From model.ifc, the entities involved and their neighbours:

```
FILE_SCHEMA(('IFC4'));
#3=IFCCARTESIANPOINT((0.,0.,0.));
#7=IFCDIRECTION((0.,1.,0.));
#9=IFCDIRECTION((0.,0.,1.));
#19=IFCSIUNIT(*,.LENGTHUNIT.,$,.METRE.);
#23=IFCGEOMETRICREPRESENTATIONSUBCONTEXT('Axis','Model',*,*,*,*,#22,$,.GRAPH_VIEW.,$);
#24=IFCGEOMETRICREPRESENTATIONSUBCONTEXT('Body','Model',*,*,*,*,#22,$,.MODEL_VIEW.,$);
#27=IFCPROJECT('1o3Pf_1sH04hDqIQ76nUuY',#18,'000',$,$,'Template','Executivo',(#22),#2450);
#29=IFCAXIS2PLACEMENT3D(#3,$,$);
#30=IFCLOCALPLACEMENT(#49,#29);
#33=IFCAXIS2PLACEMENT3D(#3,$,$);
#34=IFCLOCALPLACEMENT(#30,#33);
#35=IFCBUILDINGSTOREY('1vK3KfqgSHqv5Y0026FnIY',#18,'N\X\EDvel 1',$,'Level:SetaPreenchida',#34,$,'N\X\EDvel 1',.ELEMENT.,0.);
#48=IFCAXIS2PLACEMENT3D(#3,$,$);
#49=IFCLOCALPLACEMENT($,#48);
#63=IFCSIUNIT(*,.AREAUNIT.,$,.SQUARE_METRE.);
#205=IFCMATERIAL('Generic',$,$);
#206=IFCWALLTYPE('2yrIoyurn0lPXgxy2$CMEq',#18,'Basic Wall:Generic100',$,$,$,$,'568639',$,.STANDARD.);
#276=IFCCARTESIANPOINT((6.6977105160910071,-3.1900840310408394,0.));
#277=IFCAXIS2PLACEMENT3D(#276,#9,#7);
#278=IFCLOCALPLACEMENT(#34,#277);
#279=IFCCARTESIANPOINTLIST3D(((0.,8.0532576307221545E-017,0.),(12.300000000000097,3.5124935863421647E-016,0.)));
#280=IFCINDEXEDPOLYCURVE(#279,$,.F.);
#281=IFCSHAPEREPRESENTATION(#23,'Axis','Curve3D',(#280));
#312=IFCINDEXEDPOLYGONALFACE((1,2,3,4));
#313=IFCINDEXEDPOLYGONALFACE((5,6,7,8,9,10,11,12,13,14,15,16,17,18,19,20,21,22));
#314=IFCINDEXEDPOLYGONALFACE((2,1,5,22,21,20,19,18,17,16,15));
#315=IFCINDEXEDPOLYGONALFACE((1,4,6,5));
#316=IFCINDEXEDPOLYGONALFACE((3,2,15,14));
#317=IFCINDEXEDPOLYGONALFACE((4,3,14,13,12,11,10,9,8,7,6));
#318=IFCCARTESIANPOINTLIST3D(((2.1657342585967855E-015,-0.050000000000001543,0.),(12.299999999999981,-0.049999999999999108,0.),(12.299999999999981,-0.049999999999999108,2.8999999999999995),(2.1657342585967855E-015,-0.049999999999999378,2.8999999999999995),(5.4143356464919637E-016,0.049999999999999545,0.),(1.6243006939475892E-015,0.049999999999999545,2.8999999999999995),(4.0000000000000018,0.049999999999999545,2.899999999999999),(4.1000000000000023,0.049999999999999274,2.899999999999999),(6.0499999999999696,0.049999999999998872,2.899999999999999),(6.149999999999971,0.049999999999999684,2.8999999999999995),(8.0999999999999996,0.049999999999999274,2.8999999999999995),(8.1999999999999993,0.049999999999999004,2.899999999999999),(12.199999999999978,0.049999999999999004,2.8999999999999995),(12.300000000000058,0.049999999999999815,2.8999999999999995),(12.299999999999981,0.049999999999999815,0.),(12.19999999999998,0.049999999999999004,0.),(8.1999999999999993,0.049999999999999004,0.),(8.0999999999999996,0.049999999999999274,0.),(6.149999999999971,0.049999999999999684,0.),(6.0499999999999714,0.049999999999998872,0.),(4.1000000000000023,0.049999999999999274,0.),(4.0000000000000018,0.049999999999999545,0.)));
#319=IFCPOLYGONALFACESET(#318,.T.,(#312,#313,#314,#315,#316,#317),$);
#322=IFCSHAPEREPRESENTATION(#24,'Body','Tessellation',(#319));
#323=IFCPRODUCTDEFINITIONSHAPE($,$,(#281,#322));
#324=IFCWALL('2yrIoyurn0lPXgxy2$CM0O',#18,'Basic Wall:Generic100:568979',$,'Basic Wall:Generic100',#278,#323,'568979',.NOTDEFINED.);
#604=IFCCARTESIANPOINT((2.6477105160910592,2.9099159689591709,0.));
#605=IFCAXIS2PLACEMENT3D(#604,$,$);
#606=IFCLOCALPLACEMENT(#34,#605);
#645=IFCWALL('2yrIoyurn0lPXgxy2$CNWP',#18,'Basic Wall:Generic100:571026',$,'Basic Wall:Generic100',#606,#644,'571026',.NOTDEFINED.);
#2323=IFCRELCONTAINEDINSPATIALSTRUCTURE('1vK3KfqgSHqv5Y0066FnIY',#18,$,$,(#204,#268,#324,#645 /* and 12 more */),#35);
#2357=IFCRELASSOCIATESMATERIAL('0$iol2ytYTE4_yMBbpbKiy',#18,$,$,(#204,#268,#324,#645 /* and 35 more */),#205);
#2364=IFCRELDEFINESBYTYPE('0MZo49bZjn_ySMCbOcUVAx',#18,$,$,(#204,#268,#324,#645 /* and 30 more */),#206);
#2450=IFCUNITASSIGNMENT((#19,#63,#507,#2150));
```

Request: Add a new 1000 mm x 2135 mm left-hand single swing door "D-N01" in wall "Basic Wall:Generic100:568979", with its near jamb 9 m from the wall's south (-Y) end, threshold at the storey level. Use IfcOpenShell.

```python
import numpy as np
import ifcopenshell
import ifcopenshell.api.feature
import ifcopenshell.api.geometry
import ifcopenshell.api.root
import ifcopenshell.api.spatial
import ifcopenshell.geom
import ifcopenshell.util.element
import ifcopenshell.util.placement
import ifcopenshell.util.representation
import ifcopenshell.util.shape
import ifcopenshell.util.unit

model = ifcopenshell.open("model.ifc")
unit_scale = ifcopenshell.util.unit.calculate_unit_scale(model)
settings = ifcopenshell.geom.settings()


def volume(element):
    """Net volume in cubic metres, openings subtracted."""
    shape = ifcopenshell.geom.create_shape(settings, element)
    return ifcopenshell.util.shape.get_volume(shape.geometry)


wall = model.by_guid("2yrIoyurn0lPXgxy2$CM0O")
storey = ifcopenshell.util.element.get_container(wall, ifc_class="IfcBuildingStorey")
context = ifcopenshell.util.representation.get_context(model, "Model", "Body", "MODEL_VIEW")
before = volume(wall)

width, height, from_end, sill = 1, 2.135, 9, 0.0  # metres

# The wall runs along its own X axis, and the end named is its -X end.
wall_shape = ifcopenshell.geom.create_shape(settings, wall)
x, y, z = ifcopenshell.util.shape.get_vertices(wall_shape.geometry).T
start = x.min() + from_end
face, thickness = float(y.min()), float(y.max() - y.min())
wall_matrix = ifcopenshell.util.placement.get_local_placement(wall.ObjectPlacement)
level = ifcopenshell.util.placement.get_local_placement(storey.ObjectPlacement)[2, 3]


def in_wall(x, y):
    """Placement at x, y metres in the wall's axes, at sill height."""
    matrix = wall_matrix.copy()
    matrix[:, 3] = wall_matrix @ np.array([x / unit_scale, y / unit_scale, 0.0, 1.0])
    matrix[2, 3] = level + sill / unit_scale
    return matrix


# Opening: a box that overshoots both wall faces by 50 mm.
opening = ifcopenshell.api.root.create_entity(model, ifc_class="IfcOpeningElement", predefined_type="OPENING")
box = ifcopenshell.api.geometry.add_wall_representation(
    model, context=context, length=width, height=height, thickness=thickness + 0.1
)
ifcopenshell.api.geometry.assign_representation(model, product=opening, representation=box)
ifcopenshell.api.geometry.edit_object_placement(model, product=opening, matrix=in_wall(start, face - 0.05), is_si=False)
ifcopenshell.api.feature.add_feature(model, feature=opening, element=wall)

door = ifcopenshell.api.root.create_entity(model, ifc_class="IfcDoor", name="D-N01", predefined_type="DOOR")
door.OverallWidth, door.OverallHeight = width / unit_scale, height / unit_scale
door.OperationType = "SINGLE_SWING_LEFT"
body = ifcopenshell.api.geometry.add_door_representation(
    model,
    context=context,
    overall_width=door.OverallWidth,
    overall_height=door.OverallHeight,
    operation_type="SINGLE_SWING_LEFT",
    lining_properties={"LiningDepth": thickness / unit_scale, "ThresholdDepth": thickness / unit_scale},
)
ifcopenshell.api.geometry.assign_representation(model, product=door, representation=body)
ifcopenshell.api.spatial.assign_container(model, products=[door], relating_structure=storey)
ifcopenshell.api.feature.add_filling(model, opening=opening, element=door)

# The lining spans the wall, so the door starts at the wall face.
ifcopenshell.api.geometry.edit_object_placement(model, product=door, matrix=in_wall(start, face), is_si=False)

after = volume(wall)

print(f"wall volume {before:.3f} -> {after:.3f} m3")

model.write("model_v2.ifc")
```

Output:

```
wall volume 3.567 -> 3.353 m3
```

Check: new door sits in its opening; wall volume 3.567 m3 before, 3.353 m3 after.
